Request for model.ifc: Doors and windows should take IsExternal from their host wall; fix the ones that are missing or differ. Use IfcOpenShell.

First a look at what the model holds.

```python
import ifcopenshell
import ifcopenshell.util.element

model = ifcopenshell.open("model.ifc")
print(model.schema)
seen = {}
for e in model.by_type("IfcDoor") + model.by_type("IfcWindow"):
    if not e.FillsVoids:
        continue
    host = e.FillsVoids[0].RelatingOpeningElement.VoidsElements[0].RelatingBuildingElement
    own = ifcopenshell.util.element.get_pset(e, f"Pset_{e.is_a()[3:].removesuffix('StandardCase')}Common", "IsExternal")
    wall = ifcopenshell.util.element.get_pset(host, "Pset_WallCommon", "IsExternal")
    seen[e.is_a(), own, wall] = seen.get((e.is_a(), own, wall), 0) + 1
for (cls, own, wall), count in sorted(seen.items(), key=str):
    print(count, cls, "IsExternal:", own, "| host wall:", wall)
```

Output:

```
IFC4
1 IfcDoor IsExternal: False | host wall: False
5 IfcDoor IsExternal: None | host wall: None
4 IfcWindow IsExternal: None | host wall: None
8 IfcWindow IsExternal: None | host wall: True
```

```python
import ifcopenshell
import ifcopenshell.api.pset
import ifcopenshell.util.element

model = ifcopenshell.open("model.ifc")

count = 0
for ifc_class, pset_name in (("IfcDoor", "Pset_DoorCommon"), ("IfcWindow", "Pset_WindowCommon")):
    for e in model.by_type(ifc_class):
        if not e.FillsVoids:
            continue
        host = e.FillsVoids[0].RelatingOpeningElement.VoidsElements[0].RelatingBuildingElement
        external = ifcopenshell.util.element.get_pset(host, "Pset_WallCommon", "IsExternal")
        if external is None or ifcopenshell.util.element.get_pset(e, pset_name, "IsExternal") == external:
            continue
        pset = ifcopenshell.api.pset.add_pset(model, product=e, name=pset_name)
        ifcopenshell.api.pset.edit_pset(model, pset=pset, properties={"IsExternal": external})
        count += 1

print(count, "updated")

model.write("model_v2.ifc")
```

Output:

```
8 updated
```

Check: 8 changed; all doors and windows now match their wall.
